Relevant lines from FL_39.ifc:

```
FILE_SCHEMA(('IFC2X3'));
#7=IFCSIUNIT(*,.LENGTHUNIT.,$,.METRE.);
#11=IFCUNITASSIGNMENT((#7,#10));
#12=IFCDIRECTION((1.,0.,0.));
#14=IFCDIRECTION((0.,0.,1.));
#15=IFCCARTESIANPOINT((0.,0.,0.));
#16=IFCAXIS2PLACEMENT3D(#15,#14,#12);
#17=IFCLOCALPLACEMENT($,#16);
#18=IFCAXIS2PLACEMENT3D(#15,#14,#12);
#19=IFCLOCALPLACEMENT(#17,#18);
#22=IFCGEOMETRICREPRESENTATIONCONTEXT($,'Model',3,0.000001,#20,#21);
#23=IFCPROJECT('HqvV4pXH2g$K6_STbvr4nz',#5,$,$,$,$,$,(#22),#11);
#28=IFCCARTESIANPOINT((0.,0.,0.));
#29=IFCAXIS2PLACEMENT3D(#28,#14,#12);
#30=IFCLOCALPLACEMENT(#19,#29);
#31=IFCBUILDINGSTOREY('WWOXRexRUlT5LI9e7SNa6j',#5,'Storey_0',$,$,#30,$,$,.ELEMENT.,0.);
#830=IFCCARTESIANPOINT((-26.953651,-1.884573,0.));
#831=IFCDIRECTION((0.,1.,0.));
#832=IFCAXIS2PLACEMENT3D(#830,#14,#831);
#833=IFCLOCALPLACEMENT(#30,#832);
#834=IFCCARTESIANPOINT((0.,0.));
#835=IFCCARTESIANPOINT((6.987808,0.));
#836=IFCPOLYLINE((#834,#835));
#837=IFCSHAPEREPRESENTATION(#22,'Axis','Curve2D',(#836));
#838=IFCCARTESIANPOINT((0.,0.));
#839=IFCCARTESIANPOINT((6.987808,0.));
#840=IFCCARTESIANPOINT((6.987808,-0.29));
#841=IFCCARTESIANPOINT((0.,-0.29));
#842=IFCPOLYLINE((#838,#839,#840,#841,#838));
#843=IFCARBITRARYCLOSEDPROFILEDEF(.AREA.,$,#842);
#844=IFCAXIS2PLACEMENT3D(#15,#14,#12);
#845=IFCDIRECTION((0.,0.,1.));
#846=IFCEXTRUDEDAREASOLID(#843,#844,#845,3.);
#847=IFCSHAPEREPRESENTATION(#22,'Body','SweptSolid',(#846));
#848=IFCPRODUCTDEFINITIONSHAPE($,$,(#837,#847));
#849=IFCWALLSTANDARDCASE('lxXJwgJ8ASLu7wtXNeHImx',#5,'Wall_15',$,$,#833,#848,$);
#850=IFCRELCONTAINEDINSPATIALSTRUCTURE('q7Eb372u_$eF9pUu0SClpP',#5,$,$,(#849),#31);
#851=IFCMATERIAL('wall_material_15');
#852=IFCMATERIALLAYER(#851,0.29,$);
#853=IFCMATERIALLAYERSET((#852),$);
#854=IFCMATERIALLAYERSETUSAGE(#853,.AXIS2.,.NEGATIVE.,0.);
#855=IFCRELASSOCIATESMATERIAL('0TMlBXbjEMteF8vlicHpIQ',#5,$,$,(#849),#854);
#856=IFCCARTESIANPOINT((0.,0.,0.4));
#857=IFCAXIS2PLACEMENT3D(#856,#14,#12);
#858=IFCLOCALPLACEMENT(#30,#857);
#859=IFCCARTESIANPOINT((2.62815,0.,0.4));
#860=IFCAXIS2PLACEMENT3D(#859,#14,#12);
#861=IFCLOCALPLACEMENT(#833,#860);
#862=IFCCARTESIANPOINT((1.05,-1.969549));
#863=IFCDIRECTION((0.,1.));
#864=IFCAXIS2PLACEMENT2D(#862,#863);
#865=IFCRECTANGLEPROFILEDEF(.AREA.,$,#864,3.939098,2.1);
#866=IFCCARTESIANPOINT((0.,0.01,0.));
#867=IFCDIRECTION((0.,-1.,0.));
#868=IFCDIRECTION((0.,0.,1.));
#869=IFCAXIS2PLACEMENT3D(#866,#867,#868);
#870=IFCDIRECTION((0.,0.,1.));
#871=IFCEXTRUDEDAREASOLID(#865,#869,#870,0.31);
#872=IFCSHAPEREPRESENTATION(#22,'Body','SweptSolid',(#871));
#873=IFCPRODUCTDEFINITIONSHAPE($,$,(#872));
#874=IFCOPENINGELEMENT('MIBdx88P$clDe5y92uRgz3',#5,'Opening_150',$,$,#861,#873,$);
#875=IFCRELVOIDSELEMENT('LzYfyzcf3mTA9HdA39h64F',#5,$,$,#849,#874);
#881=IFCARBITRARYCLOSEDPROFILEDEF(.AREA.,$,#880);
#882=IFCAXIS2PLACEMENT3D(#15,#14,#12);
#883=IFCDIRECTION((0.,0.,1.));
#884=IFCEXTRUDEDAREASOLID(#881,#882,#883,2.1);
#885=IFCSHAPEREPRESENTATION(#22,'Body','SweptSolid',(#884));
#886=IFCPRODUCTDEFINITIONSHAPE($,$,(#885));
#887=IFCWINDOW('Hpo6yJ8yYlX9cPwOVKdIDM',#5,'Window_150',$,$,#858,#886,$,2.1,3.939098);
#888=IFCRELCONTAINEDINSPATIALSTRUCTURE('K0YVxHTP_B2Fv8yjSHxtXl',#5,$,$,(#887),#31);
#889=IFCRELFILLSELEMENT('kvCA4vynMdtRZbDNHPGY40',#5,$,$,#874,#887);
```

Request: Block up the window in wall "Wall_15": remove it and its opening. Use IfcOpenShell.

```python
import ifcopenshell
import ifcopenshell.api.feature
import ifcopenshell.api.root
import ifcopenshell.geom
import ifcopenshell.util.shape

model = ifcopenshell.open("FL_39.ifc")
settings = ifcopenshell.geom.settings()


def volume(element):
    """Net volume in cubic metres, openings subtracted."""
    shape = ifcopenshell.geom.create_shape(settings, element)
    return ifcopenshell.util.shape.get_volume(shape.geometry)


window = model.by_id(887)
opening = window.FillsVoids[0].RelatingOpeningElement
wall = opening.VoidsElements[0].RelatingBuildingElement
before = volume(wall)

ifcopenshell.api.root.remove_product(model, product=window)
ifcopenshell.api.feature.remove_feature(model, feature=opening)

after = volume(wall)

print(f"wall volume {before:.3f} -> {after:.3f} m3")

model.write("FL_39-out.ifc")
```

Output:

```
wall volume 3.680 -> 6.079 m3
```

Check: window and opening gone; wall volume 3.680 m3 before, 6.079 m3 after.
